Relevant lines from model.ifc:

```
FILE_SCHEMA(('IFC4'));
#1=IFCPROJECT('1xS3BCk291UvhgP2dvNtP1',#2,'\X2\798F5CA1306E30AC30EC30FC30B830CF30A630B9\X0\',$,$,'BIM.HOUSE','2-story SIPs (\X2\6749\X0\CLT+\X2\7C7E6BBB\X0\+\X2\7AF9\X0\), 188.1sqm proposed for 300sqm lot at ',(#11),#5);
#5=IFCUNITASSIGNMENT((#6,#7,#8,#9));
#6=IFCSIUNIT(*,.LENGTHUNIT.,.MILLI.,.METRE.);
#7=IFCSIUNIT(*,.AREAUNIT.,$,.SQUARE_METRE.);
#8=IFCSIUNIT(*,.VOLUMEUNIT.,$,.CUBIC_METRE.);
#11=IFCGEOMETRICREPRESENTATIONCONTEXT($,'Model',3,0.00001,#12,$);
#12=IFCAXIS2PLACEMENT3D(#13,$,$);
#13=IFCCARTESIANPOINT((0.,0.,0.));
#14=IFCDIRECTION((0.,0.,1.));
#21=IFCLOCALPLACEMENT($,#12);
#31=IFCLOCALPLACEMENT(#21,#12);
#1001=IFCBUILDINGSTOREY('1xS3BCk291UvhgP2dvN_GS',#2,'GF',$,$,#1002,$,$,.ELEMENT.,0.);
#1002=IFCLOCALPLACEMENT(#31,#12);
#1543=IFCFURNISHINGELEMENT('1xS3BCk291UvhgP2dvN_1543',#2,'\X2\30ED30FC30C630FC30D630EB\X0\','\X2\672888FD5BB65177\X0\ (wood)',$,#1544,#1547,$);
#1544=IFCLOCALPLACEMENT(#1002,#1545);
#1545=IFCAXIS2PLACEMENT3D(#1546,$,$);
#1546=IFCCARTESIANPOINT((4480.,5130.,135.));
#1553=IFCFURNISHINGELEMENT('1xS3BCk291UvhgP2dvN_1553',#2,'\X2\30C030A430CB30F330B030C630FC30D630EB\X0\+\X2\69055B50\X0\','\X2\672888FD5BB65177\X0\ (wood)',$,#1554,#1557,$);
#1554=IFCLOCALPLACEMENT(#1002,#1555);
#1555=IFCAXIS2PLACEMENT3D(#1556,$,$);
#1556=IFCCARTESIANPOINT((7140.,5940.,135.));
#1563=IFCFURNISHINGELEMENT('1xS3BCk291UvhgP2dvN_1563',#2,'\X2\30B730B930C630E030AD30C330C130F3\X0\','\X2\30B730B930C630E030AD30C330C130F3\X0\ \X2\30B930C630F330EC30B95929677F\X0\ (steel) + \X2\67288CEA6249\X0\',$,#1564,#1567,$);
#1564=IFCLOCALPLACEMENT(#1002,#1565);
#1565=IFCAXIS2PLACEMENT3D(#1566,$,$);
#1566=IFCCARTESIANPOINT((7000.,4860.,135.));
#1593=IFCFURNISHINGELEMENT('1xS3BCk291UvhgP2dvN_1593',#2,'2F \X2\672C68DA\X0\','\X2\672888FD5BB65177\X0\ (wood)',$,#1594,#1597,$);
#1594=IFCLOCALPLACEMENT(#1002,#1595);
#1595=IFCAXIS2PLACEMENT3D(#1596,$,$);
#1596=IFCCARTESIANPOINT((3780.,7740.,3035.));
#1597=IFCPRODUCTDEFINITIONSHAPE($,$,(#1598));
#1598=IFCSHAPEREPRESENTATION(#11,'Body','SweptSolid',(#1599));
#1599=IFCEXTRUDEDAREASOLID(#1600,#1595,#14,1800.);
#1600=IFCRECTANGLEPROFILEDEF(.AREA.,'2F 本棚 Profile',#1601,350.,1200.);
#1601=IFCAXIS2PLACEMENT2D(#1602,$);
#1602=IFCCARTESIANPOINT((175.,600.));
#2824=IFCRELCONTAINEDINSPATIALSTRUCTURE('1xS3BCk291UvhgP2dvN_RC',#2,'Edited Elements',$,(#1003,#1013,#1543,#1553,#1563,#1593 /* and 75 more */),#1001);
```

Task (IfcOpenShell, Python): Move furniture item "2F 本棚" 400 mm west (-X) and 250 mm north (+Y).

```python
import ifcopenshell
import ifcopenshell.api.geometry
import ifcopenshell.util.placement

model = ifcopenshell.open("model.ifc")

item = model.by_id(1593)
matrix = ifcopenshell.util.placement.get_local_placement(item.ObjectPlacement)
matrix[0, 3] -= 400.0
matrix[1, 3] += 250.0
ifcopenshell.api.geometry.edit_object_placement(model, product=item, matrix=matrix, is_si=False)

print(ifcopenshell.util.placement.get_local_placement(item.ObjectPlacement).round(3) + 0.0)

model.write("model_updated.ifc")
```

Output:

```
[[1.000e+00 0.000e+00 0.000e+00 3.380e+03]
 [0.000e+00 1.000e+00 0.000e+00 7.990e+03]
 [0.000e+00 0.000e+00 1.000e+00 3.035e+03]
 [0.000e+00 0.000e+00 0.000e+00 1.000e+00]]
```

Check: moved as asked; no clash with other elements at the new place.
